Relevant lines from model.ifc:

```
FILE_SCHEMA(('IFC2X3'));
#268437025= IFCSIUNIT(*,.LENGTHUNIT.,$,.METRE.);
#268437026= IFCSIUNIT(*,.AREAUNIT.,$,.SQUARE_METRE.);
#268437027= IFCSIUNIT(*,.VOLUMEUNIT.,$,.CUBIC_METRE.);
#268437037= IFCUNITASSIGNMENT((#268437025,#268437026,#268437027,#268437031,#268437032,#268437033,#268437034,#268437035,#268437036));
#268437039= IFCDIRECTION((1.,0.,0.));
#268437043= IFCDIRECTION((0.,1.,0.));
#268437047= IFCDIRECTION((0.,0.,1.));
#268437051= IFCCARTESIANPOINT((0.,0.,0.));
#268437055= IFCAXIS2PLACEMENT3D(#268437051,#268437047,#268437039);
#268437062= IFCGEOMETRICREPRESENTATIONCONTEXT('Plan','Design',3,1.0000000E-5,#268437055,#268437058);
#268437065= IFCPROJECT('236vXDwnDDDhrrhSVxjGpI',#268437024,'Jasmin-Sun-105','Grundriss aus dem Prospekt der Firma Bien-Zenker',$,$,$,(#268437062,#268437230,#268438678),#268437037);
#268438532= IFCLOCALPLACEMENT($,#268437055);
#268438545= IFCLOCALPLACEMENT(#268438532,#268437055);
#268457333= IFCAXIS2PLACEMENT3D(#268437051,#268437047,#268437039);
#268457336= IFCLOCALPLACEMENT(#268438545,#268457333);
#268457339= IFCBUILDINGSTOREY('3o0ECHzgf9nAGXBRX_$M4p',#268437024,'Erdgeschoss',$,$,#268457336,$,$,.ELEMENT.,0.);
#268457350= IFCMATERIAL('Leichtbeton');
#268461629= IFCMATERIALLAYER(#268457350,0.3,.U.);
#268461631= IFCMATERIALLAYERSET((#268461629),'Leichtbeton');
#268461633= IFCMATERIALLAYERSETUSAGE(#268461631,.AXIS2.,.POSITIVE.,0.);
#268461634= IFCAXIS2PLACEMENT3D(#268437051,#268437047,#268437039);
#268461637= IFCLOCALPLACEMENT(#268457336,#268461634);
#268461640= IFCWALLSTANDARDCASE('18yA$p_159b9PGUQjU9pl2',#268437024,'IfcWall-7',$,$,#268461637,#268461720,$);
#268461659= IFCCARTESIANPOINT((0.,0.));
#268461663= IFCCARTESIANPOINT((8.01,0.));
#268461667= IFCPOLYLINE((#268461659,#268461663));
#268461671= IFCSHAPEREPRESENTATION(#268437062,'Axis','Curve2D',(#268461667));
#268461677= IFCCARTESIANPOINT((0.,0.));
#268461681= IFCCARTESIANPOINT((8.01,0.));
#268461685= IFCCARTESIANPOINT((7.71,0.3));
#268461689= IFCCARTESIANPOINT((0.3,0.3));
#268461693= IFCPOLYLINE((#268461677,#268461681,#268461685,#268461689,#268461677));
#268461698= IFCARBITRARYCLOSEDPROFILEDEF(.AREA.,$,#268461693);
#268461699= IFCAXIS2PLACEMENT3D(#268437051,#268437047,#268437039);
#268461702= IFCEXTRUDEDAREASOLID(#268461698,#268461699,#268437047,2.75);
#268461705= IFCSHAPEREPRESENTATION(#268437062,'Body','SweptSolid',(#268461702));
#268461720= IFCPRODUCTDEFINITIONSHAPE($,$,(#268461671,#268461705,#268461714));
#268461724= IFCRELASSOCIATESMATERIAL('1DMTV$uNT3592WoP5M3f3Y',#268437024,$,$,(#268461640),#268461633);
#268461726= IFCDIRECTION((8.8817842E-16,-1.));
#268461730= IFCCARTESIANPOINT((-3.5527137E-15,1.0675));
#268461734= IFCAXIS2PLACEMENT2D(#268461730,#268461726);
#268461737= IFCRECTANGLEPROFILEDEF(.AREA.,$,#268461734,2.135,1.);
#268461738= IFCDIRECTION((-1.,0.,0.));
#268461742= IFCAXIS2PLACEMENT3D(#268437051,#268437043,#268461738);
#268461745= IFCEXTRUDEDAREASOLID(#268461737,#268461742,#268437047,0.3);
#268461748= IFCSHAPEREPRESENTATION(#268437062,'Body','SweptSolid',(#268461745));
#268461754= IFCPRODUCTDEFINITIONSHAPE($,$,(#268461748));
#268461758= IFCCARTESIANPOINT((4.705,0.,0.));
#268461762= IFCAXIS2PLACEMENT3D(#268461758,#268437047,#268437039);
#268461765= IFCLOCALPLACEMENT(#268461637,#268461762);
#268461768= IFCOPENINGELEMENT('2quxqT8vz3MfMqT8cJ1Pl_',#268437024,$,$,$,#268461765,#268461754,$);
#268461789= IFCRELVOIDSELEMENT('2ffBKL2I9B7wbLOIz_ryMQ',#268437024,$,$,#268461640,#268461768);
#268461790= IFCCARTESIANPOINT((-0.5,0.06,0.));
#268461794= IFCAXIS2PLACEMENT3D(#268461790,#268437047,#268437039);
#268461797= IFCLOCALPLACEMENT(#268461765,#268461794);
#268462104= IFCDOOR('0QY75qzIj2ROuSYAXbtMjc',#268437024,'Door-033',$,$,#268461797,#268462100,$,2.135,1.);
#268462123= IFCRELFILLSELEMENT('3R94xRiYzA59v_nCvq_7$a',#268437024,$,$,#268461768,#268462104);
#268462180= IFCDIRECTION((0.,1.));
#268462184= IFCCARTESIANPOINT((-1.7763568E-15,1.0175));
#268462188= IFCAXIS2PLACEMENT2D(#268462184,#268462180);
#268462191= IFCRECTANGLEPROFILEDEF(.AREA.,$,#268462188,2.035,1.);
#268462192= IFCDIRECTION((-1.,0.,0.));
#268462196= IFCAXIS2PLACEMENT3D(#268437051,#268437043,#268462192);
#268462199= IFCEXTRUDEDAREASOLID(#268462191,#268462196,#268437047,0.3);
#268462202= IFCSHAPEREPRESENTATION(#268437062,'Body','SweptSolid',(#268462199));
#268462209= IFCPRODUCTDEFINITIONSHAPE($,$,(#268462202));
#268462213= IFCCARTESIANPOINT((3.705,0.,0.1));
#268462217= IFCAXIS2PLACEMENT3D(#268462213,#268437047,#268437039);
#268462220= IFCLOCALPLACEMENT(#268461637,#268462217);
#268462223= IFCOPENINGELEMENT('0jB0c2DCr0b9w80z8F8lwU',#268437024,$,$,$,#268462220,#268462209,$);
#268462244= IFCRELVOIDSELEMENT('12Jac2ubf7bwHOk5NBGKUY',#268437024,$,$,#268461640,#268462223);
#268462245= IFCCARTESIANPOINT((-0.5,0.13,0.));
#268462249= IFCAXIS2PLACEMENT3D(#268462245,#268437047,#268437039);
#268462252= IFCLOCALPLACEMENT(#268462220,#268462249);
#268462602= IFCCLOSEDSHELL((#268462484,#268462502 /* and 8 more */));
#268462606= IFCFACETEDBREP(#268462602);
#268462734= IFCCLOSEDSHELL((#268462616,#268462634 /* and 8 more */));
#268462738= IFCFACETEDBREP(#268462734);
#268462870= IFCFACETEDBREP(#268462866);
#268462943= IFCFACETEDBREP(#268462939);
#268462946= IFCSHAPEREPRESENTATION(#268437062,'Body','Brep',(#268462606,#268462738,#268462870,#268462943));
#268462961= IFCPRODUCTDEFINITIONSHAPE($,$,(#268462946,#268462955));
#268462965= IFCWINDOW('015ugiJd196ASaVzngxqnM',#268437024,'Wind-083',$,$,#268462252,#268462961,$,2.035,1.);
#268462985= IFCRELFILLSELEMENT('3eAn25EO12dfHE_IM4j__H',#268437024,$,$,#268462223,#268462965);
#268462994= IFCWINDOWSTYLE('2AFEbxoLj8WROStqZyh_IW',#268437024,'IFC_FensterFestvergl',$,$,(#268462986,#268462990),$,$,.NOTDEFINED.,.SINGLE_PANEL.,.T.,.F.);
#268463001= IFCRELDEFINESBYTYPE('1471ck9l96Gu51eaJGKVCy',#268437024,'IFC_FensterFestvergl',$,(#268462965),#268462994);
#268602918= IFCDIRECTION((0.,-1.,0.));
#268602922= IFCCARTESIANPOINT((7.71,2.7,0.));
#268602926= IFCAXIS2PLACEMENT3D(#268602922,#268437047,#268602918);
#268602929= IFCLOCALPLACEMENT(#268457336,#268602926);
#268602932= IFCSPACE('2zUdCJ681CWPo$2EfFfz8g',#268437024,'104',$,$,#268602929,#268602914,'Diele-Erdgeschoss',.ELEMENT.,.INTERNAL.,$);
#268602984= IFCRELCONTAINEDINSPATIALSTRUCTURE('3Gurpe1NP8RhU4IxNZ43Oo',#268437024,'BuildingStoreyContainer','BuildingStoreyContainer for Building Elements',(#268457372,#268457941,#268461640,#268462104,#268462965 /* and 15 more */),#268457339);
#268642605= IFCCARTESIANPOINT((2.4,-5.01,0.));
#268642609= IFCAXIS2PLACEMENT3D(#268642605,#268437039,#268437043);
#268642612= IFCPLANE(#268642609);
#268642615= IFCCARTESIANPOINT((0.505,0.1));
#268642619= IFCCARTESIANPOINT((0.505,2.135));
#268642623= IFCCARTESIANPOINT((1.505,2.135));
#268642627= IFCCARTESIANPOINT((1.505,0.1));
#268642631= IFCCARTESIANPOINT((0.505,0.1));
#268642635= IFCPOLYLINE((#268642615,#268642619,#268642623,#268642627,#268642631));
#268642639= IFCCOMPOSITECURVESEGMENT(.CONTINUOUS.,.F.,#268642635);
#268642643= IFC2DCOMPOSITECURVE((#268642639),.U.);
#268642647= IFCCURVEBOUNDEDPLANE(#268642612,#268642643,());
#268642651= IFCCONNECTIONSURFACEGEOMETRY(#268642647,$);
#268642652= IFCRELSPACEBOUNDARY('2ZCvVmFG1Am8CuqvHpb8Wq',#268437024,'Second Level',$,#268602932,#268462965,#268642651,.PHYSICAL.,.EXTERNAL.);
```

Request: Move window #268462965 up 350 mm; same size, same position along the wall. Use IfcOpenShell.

```python
import numpy as np
import ifcopenshell
import ifcopenshell.api.geometry
import ifcopenshell.util.placement
import ifcopenshell.util.unit

model = ifcopenshell.open("model.ifc")
unit_scale = ifcopenshell.util.unit.calculate_unit_scale(model)

window = model.by_id(268462965)
opening = window.FillsVoids[0].RelatingOpeningElement
dz = 0.35 / unit_scale

shift = np.array([0.0, 0.0, dz])
# The window is placed relative to its opening, so it follows when the opening moves.
matrix = ifcopenshell.util.placement.get_local_placement(opening.ObjectPlacement)
matrix[:3, 3] += shift
ifcopenshell.api.geometry.edit_object_placement(
    model, product=opening, matrix=matrix, is_si=False, should_transform_children=True
)

# Space boundary surfaces are stored in each space's coordinates; move them too.
for rel in window.ProvidesBoundaries:
    if not rel.ConnectionGeometry:
        continue
    surface = rel.ConnectionGeometry.SurfaceOnRelatingElement.BasisSurface
    space_matrix = ifcopenshell.util.placement.get_local_placement(rel.RelatingSpace.ObjectPlacement)
    point = np.array(surface.Position.Location.Coordinates) + space_matrix[:3, :3].T @ shift
    surface.Position = model.createIfcAxis2Placement3D(
        model.createIfcCartesianPoint(point.tolist()), surface.Position.Axis, surface.Position.RefDirection
    )

print(f"moved by {dz * unit_scale:+.3f} m")

model.write("model_v2.ifc")
```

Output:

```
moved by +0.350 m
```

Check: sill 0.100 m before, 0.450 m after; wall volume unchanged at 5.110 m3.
